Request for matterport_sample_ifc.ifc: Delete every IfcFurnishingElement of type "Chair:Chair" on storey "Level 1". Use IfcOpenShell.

First a look at what the model holds.

```python
import ifcopenshell
import ifcopenshell.util.element

model = ifcopenshell.open("matterport_sample_ifc.ifc")
print(model.schema)
storey = next(s for s in model.by_type("IfcBuildingStorey") if s.Name == "Level 1")
furniture = [e for e in ifcopenshell.util.element.get_decomposition(storey) if e.is_a("IfcFurnishingElement")]
seen = {}
for e in furniture:
    element_type = ifcopenshell.util.element.get_type(e)
    name = element_type.Name if element_type not in (None, e) else None
    seen[name] = seen.get(name, 0) + 1
for name, count in sorted(seen.items(), key=str):
    print(count, "x", name)
```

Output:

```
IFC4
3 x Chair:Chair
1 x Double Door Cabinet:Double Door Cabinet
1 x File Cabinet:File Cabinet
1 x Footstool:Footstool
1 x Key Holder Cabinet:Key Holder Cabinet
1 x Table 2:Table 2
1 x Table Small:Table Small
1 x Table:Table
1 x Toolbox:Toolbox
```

```python
import ifcopenshell
import ifcopenshell.api.root
import ifcopenshell.util.element

model = ifcopenshell.open("matterport_sample_ifc.ifc")

storey = next(s for s in model.by_type("IfcBuildingStorey") if s.Name == "Level 1")
furniture = [e for e in ifcopenshell.util.element.get_decomposition(storey) if e.is_a("IfcFurnishingElement")]
targets = [e for e in furniture if (t := ifcopenshell.util.element.get_type(e)) not in (None, e) and t.Name == "Chair:Chair"]

for e in targets:
    ifcopenshell.api.root.remove_product(model, product=e)
print(len(targets), "removed")

model.write("matterport_sample_ifc_edited.ifc")
```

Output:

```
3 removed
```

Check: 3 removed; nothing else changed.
